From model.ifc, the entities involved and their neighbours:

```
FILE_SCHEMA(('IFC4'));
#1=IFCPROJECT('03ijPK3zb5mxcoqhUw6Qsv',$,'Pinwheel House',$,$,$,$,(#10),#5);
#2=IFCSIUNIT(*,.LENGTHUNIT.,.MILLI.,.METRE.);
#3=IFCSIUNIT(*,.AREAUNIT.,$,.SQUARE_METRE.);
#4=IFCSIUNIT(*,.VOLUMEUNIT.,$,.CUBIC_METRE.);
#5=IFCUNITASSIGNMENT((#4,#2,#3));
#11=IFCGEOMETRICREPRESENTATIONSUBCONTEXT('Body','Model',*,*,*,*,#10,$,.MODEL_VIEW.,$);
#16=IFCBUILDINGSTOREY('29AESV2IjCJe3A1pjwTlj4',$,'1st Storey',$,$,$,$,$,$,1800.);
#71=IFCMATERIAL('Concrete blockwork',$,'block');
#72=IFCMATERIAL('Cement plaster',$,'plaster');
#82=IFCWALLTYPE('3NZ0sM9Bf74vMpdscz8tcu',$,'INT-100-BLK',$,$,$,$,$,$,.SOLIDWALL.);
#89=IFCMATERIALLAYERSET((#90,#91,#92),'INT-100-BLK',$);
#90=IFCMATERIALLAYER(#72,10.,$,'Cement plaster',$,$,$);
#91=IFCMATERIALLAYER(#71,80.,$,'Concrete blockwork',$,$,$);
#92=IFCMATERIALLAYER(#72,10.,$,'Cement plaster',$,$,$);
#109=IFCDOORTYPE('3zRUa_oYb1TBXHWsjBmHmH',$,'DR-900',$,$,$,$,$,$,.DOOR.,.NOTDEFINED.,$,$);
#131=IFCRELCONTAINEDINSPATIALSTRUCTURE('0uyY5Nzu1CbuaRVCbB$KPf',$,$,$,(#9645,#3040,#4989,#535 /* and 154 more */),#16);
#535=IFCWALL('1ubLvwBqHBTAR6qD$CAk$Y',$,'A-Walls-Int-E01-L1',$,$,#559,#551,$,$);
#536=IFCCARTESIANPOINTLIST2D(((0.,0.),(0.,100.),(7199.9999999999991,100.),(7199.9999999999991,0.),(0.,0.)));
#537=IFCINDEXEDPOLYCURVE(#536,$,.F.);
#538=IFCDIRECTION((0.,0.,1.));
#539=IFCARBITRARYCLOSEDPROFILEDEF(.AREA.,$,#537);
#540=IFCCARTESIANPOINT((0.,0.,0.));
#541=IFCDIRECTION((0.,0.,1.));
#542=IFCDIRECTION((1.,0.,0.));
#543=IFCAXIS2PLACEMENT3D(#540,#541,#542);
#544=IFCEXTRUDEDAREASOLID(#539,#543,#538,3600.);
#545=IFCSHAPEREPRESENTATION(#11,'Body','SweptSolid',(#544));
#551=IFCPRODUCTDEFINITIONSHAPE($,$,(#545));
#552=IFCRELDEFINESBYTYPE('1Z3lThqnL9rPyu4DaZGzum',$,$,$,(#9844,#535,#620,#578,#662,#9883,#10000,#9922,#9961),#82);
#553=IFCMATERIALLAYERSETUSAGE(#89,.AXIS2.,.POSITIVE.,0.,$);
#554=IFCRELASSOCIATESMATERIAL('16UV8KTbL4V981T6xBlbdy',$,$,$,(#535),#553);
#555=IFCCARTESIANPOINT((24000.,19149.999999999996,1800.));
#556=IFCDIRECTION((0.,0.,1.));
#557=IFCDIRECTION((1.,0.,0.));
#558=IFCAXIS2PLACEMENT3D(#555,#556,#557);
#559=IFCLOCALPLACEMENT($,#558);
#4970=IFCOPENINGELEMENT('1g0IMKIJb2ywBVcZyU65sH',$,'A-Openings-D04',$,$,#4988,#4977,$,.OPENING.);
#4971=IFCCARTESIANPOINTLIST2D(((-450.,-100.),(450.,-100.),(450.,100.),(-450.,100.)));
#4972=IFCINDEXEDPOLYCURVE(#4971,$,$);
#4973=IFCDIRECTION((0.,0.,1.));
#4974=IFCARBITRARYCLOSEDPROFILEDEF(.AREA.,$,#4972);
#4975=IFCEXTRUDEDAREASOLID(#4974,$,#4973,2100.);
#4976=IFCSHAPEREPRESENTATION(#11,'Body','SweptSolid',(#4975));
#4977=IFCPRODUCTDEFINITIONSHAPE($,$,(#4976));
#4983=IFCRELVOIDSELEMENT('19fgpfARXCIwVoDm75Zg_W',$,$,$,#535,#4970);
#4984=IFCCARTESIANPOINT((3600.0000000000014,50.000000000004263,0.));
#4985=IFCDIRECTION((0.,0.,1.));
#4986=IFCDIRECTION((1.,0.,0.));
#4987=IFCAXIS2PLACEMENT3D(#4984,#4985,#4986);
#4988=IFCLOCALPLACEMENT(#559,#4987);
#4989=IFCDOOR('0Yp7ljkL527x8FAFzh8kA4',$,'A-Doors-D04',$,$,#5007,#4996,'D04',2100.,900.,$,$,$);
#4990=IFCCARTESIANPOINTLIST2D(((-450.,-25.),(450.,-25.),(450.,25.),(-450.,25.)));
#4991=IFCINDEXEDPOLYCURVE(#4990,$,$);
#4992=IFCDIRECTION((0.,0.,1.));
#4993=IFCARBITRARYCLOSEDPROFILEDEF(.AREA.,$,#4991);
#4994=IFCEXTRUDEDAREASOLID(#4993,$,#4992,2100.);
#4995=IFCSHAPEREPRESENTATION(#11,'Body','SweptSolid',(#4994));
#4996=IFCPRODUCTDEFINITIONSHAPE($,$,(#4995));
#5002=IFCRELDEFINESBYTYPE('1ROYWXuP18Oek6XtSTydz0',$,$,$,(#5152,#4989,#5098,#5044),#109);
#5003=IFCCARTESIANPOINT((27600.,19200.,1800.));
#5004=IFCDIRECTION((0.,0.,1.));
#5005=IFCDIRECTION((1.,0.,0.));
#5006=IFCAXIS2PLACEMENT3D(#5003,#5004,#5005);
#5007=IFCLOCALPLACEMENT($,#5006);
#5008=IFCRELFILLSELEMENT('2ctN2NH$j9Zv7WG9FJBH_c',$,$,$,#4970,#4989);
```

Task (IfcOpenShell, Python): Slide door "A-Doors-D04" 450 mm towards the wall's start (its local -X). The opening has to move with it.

```python
import ifcopenshell
import ifcopenshell.api.geometry
import ifcopenshell.util.placement

model = ifcopenshell.open("model.ifc")

door = model.by_guid("0Yp7ljkL527x8FAFzh8kA4")
opening = door.FillsVoids[0].RelatingOpeningElement
wall = opening.VoidsElements[0].RelatingBuildingElement

wall_matrix = ifcopenshell.util.placement.get_local_placement(wall.ObjectPlacement)
shift = wall_matrix[:3, 0] * -450.0
before = ifcopenshell.util.placement.get_local_placement(door.ObjectPlacement)[:3, 3].copy()

# The door is not placed relative to its opening, so move both.
for product in (opening, door):
    matrix = ifcopenshell.util.placement.get_local_placement(product.ObjectPlacement)
    matrix[:3, 3] += shift
    ifcopenshell.api.geometry.edit_object_placement(model, product=product, matrix=matrix, is_si=False)

after = ifcopenshell.util.placement.get_local_placement(door.ObjectPlacement)[:3, 3]
print("door moved by", (after - before).round(3) + 0.0)

model.write("model_v2.ifc")
```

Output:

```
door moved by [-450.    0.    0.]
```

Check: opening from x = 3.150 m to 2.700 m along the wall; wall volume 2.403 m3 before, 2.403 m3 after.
